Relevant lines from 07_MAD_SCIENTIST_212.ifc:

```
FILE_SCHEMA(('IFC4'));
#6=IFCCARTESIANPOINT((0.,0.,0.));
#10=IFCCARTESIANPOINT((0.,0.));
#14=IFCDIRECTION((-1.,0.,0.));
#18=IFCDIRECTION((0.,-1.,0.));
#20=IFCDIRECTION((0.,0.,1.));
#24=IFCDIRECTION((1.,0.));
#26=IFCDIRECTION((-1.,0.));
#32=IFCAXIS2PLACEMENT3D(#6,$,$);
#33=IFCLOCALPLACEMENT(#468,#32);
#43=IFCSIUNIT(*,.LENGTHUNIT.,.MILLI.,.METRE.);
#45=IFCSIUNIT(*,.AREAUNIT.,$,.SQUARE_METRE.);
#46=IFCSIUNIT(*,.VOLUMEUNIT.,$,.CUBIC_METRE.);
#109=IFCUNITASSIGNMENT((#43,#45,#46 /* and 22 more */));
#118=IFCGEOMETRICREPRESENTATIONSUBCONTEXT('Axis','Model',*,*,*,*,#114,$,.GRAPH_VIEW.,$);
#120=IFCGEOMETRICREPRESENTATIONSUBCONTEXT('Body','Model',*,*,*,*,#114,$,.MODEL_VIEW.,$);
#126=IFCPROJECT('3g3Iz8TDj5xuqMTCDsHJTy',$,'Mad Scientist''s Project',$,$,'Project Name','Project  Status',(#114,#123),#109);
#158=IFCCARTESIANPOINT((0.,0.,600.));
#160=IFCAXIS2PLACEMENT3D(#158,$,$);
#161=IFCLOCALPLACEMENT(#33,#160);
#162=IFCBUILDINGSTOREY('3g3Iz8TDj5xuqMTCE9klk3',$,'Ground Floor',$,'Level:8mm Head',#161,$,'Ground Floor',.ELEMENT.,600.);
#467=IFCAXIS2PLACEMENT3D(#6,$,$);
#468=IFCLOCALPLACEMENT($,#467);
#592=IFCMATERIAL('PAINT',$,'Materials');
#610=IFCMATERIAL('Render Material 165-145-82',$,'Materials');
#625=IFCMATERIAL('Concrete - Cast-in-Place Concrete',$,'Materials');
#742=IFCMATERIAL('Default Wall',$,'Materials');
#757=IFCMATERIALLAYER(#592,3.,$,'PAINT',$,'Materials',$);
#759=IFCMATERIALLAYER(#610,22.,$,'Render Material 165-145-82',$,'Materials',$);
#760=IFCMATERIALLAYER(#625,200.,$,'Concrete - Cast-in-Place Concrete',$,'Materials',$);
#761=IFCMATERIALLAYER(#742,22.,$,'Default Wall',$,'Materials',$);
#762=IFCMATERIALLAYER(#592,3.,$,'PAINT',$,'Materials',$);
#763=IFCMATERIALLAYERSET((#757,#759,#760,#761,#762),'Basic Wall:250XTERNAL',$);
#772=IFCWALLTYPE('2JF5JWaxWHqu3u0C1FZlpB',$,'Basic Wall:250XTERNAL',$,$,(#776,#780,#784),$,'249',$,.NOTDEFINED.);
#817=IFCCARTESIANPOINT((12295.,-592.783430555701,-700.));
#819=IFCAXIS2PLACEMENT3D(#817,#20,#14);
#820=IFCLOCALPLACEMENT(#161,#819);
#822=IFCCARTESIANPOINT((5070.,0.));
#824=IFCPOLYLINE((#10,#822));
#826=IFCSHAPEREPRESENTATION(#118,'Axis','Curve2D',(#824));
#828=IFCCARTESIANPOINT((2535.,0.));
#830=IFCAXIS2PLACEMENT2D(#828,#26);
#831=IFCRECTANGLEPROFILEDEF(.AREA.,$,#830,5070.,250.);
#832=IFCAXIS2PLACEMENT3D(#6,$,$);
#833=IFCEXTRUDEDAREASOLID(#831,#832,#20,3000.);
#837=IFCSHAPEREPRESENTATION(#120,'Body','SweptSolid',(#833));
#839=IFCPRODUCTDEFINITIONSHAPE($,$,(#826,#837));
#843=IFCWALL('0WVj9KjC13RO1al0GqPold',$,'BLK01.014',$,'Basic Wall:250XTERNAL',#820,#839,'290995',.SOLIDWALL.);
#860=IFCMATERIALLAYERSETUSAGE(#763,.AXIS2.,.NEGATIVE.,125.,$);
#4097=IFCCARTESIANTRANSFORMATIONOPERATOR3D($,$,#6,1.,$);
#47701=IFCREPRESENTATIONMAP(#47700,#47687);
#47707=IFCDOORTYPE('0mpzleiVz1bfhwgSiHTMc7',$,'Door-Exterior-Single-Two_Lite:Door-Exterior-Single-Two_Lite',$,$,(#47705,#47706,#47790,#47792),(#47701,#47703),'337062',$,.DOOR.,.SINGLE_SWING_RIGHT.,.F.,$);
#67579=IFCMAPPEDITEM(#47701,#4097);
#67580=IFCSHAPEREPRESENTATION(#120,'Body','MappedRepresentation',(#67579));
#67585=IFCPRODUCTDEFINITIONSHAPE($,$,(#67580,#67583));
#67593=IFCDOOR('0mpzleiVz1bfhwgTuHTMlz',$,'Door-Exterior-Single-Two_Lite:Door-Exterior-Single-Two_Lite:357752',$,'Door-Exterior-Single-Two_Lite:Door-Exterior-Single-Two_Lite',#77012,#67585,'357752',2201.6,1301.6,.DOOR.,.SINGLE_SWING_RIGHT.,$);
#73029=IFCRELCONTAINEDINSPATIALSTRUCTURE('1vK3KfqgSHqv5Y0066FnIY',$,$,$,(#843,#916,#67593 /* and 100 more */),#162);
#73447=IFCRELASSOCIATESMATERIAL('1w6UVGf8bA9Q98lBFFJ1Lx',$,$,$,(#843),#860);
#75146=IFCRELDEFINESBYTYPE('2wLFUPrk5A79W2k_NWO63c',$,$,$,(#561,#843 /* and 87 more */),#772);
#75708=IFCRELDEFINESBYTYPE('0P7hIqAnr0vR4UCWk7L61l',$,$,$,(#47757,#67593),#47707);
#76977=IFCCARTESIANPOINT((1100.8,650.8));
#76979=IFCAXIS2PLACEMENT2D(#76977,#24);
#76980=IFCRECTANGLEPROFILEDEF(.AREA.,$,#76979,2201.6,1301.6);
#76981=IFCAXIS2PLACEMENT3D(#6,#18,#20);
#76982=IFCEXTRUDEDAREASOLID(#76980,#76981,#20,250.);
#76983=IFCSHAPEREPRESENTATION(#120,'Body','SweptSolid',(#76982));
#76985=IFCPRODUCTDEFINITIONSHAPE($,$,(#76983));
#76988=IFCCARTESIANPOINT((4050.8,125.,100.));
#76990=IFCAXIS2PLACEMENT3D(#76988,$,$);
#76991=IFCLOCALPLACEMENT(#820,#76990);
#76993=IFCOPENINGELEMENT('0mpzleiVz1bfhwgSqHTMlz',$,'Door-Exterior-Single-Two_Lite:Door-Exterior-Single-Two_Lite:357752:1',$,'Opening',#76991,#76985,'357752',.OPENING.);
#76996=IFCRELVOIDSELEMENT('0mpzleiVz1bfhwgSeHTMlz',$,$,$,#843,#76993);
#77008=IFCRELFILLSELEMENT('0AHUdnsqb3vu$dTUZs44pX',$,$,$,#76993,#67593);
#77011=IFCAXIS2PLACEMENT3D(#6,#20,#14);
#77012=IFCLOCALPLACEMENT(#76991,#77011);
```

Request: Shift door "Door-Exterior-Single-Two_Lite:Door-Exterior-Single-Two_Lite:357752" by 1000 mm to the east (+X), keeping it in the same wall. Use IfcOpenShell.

```python
import ifcopenshell
import ifcopenshell.api.geometry
import ifcopenshell.util.placement

model = ifcopenshell.open("07_MAD_SCIENTIST_212.ifc")

door = model.by_id(67593)
opening = door.FillsVoids[0].RelatingOpeningElement
wall = opening.VoidsElements[0].RelatingBuildingElement

wall_matrix = ifcopenshell.util.placement.get_local_placement(wall.ObjectPlacement)
shift = wall_matrix[:3, 0] * -1000.0
before = ifcopenshell.util.placement.get_local_placement(door.ObjectPlacement)[:3, 3].copy()

# The door is placed relative to its opening, so it follows when the opening moves.
matrix = ifcopenshell.util.placement.get_local_placement(opening.ObjectPlacement)
matrix[:3, 3] += shift
ifcopenshell.api.geometry.edit_object_placement(
    model, product=opening, matrix=matrix, is_si=False, should_transform_children=True
)

after = ifcopenshell.util.placement.get_local_placement(door.ObjectPlacement)[:3, 3]
print("door moved by", (after - before).round(3) + 0.0)

model.write("07_MAD_SCIENTIST_212_rev.ifc")
```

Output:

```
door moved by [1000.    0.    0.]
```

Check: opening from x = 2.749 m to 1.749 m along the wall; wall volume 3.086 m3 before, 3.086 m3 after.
